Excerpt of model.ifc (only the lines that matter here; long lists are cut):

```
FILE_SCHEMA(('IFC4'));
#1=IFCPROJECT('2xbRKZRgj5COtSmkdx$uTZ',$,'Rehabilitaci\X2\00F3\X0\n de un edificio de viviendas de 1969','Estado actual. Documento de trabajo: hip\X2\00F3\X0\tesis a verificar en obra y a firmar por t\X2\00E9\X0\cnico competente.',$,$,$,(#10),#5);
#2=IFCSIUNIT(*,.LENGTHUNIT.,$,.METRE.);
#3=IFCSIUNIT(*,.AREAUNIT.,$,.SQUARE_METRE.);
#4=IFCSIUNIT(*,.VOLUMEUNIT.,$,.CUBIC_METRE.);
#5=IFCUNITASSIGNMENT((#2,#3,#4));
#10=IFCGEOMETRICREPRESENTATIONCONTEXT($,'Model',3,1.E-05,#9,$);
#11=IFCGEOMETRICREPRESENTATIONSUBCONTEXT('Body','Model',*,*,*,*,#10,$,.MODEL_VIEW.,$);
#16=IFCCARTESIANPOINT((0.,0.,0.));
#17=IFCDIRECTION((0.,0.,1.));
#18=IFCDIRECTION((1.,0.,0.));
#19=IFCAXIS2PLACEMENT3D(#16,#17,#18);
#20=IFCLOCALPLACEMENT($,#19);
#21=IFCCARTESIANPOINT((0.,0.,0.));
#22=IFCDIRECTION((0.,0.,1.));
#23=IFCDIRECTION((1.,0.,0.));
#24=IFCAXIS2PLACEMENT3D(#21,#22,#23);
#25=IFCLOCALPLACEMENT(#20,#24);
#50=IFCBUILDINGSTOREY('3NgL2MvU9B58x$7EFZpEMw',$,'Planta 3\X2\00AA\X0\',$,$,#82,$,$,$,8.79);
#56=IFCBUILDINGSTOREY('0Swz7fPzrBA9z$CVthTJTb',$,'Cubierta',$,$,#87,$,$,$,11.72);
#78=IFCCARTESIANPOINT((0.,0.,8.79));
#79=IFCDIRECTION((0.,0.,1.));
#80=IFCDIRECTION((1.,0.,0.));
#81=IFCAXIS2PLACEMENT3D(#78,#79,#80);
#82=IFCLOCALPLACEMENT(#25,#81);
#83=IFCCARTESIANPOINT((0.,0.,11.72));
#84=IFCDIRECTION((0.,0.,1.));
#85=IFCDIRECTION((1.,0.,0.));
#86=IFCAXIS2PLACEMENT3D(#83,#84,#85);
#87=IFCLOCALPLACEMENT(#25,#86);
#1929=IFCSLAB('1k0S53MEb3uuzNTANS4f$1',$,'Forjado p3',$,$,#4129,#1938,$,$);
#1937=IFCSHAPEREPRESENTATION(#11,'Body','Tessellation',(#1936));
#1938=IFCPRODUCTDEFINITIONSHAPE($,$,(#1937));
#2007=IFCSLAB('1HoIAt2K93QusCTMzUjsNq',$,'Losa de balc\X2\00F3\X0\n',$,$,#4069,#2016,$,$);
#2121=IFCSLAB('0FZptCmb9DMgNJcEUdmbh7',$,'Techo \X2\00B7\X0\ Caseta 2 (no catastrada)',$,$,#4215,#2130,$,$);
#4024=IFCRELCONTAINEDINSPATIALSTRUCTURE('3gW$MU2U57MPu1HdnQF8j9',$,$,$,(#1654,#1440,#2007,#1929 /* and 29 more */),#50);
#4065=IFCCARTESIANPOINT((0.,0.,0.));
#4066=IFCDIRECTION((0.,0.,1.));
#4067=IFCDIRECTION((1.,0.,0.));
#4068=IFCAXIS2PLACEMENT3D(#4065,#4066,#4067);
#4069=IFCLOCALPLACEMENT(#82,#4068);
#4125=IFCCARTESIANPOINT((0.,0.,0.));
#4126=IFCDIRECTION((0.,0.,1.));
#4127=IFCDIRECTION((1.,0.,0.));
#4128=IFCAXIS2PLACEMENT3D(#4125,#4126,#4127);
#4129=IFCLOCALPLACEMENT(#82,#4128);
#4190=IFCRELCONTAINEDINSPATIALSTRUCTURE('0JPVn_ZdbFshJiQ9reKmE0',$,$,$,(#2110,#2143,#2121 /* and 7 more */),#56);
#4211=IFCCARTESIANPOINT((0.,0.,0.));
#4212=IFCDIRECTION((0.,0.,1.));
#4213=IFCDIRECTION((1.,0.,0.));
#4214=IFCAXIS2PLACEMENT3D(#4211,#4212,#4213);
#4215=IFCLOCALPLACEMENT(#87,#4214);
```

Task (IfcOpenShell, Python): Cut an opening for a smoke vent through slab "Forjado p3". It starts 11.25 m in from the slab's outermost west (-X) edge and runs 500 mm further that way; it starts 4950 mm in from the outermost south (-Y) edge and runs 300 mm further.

```python
import numpy as np
import ifcopenshell
import ifcopenshell.api.feature
import ifcopenshell.api.geometry
import ifcopenshell.api.root
import ifcopenshell.geom
import ifcopenshell.util.placement
import ifcopenshell.util.representation
import ifcopenshell.util.shape
import ifcopenshell.util.unit

model = ifcopenshell.open("model.ifc")
unit_scale = ifcopenshell.util.unit.calculate_unit_scale(model)
settings = ifcopenshell.geom.settings()


def volume(element):
    """Net volume in cubic metres, openings subtracted."""
    shape = ifcopenshell.geom.create_shape(settings, element)
    return ifcopenshell.util.shape.get_volume(shape.geometry)


slab = model.by_guid("1k0S53MEb3uuzNTANS4f$1")
before = volume(slab)

# Extent in the slab's own axes, in metres. The edges named are its -X and -Y sides.
slab_shape = ifcopenshell.geom.create_shape(settings, slab)
vertices = ifcopenshell.util.shape.get_vertices(slab_shape.geometry)
x_min, y_min, bottom = vertices.min(axis=0)
top = vertices[:, 2].max()

opening = ifcopenshell.api.root.create_entity(model, ifc_class="IfcOpeningElement", name="Smoke vent opening", predefined_type="OPENING")
context = ifcopenshell.util.representation.get_context(model, "Model", "Body", "MODEL_VIEW")
width, depth = 0.5, 0.3
outline = [(0.0, 0.0), (width, 0.0), (width, depth), (0.0, depth), (0.0, 0.0)]
# Overshoot both faces by 50 mm so the cut is clean.
shape = ifcopenshell.api.geometry.add_slab_representation(
    model, context=context, depth=top - bottom + 0.1, polyline=outline
)
ifcopenshell.api.geometry.assign_representation(model, product=opening, representation=shape)

matrix = ifcopenshell.util.placement.get_local_placement(slab.ObjectPlacement)
matrix[:, 3] = matrix @ np.append(np.array([x_min + 11.25, y_min + 4.95, bottom - 0.05]) / unit_scale, 1.0)
ifcopenshell.api.geometry.edit_object_placement(model, product=opening, matrix=matrix, is_si=False)
ifcopenshell.api.feature.add_feature(model, feature=opening, element=slab)

after = volume(slab)

print(f"slab volume {before:.3f} -> {after:.3f} m3")

model.write("model-out.ifc")
```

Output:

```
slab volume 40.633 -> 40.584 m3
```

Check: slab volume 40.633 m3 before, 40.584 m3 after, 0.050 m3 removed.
